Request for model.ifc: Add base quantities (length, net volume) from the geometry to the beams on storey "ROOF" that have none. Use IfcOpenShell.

First a look at what the model holds.

```python
import ifcopenshell
import ifcopenshell.util.element
import ifcopenshell.util.unit

model = ifcopenshell.open("model.ifc")
print(model.schema)
for unit_type in ("LENGTHUNIT", "AREAUNIT", "VOLUMEUNIT"):
    print(unit_type, ifcopenshell.util.unit.calculate_unit_scale(model, unit_type))
storey = next(s for s in model.by_type("IfcBuildingStorey") if s.Name == "ROOF")
beams = [e for e in ifcopenshell.util.element.get_decomposition(storey) if e.is_a("IfcBeam")]
for e in sorted(beams, key=lambda e: e.id()):
    print(e.id(), e.is_a(), e.Name, list(ifcopenshell.util.element.get_psets(e, qtos_only=True)), sep=" | ")
```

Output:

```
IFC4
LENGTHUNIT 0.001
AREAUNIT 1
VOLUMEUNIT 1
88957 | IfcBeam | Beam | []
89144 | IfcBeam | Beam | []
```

```python
import ifcopenshell
import ifcopenshell.api.pset
import ifcopenshell.geom
import ifcopenshell.util.element
import ifcopenshell.util.shape
import ifcopenshell.util.unit

model = ifcopenshell.open("model.ifc")
unit_scale = ifcopenshell.util.unit.calculate_unit_scale(model)
volume_scale = ifcopenshell.util.unit.calculate_unit_scale(model, "VOLUMEUNIT")
settings = ifcopenshell.geom.settings()

storey = next(s for s in model.by_type("IfcBuildingStorey") if s.Name == "ROOF")
beams = [e for e in ifcopenshell.util.element.get_decomposition(storey) if e.is_a("IfcBeam")]

for e in sorted(beams, key=lambda e: e.id()):
    if ifcopenshell.util.element.get_psets(e, qtos_only=True, should_inherit=False):
        continue
    # Geometry comes back in metres, in the element's own axes.
    shape = ifcopenshell.geom.create_shape(settings, e)
    values = {
        "Length": ifcopenshell.util.shape.get_max_xyz(shape.geometry) / unit_scale,
        "NetVolume": ifcopenshell.util.shape.get_volume(shape.geometry) / volume_scale,
    }
    qto = ifcopenshell.api.pset.add_qto(model, product=e, name="Qto_BeamBaseQuantities")
    ifcopenshell.api.pset.edit_qto(model, qto=qto, properties=values)
    print(e.id(), {k: round(v, 3) for k, v in values.items()})

model.write("model_edited.ifc")
```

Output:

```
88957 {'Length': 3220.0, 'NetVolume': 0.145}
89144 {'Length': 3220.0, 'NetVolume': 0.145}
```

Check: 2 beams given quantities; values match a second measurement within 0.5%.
